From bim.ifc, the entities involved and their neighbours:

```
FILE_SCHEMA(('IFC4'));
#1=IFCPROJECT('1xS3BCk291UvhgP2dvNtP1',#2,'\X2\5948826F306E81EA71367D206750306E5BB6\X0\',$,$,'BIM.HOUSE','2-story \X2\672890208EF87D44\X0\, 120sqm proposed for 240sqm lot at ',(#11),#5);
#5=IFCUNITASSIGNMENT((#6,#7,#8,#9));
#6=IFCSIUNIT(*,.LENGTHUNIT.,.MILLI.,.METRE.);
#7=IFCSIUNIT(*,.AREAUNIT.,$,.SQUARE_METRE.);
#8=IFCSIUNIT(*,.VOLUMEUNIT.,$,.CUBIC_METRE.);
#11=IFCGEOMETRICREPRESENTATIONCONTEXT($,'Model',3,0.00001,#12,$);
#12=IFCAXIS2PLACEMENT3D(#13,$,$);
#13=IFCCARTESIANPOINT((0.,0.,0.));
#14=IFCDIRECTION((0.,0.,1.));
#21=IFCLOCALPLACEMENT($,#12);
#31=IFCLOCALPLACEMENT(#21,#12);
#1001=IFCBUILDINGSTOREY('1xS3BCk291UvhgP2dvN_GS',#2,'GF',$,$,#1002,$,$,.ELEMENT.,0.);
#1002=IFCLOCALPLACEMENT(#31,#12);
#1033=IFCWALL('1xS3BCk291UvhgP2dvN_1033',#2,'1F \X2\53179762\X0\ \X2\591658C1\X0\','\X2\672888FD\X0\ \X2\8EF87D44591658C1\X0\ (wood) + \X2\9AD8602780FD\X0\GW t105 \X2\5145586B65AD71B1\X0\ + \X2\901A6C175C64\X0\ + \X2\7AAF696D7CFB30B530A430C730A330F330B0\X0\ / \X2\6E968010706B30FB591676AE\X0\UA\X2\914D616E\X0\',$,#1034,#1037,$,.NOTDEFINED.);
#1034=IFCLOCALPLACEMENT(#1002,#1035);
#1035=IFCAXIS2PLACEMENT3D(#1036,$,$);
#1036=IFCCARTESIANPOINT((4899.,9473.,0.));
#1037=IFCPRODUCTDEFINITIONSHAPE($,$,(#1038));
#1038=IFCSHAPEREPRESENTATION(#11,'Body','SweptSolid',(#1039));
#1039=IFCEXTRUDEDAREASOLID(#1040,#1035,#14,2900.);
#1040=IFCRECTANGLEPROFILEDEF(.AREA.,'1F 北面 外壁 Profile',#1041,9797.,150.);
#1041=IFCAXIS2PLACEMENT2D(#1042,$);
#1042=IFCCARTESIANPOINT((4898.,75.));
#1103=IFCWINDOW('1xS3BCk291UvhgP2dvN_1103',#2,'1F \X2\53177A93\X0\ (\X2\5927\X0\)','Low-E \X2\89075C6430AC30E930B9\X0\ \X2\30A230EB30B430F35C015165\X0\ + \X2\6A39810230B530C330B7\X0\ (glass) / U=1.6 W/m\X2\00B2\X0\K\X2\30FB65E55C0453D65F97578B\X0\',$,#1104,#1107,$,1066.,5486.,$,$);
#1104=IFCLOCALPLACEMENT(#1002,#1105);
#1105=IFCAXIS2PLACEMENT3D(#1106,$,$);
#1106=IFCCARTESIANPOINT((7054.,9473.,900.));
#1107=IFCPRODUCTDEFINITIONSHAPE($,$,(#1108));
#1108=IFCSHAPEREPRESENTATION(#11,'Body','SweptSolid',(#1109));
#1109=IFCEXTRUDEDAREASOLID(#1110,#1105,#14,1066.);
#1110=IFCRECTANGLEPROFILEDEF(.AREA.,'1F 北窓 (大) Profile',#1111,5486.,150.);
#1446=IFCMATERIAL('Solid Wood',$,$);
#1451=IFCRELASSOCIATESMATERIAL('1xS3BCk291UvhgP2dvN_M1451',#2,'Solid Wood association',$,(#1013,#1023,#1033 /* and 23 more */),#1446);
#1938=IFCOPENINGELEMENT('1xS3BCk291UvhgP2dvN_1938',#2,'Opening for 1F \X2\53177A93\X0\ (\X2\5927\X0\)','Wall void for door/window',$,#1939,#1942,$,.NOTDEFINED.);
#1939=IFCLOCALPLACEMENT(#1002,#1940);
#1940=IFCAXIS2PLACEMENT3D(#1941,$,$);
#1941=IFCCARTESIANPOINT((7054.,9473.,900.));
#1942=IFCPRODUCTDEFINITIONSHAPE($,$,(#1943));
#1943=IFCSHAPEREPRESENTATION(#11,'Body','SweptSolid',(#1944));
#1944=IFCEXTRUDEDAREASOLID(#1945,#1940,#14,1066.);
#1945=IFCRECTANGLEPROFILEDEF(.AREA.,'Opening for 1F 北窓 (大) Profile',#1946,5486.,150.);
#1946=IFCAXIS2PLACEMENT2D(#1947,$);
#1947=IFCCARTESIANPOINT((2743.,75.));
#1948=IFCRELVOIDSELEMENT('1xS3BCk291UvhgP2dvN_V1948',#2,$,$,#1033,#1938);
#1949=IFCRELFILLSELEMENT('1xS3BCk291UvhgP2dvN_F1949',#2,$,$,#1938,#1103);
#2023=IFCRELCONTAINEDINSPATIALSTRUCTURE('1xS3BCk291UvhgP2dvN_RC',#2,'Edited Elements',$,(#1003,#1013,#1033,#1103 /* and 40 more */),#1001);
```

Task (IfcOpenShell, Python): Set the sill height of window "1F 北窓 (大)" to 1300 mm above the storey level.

```python
import numpy as np
import ifcopenshell
import ifcopenshell.api.geometry
import ifcopenshell.geom
import ifcopenshell.util.element
import ifcopenshell.util.placement
import ifcopenshell.util.shape
import ifcopenshell.util.unit

model = ifcopenshell.open("bim.ifc")
unit_scale = ifcopenshell.util.unit.calculate_unit_scale(model)

window = model.by_id(1103)
opening = window.FillsVoids[0].RelatingOpeningElement
storey = ifcopenshell.util.element.get_container(window, ifc_class="IfcBuildingStorey")
level = ifcopenshell.util.placement.get_local_placement(storey.ObjectPlacement)[2, 3]

# The opening's origin need not be at the sill, so measure its lowest point.
shape = ifcopenshell.geom.create_shape(ifcopenshell.geom.settings(), opening)
bottom = ifcopenshell.util.shape.get_shape_bottom_elevation(shape, shape.geometry) / unit_scale
dz = level + 1.3 / unit_scale - bottom

shift = np.array([0.0, 0.0, dz])
# The window is not placed relative to its opening, so move both.
for product in (opening, window):
    matrix = ifcopenshell.util.placement.get_local_placement(product.ObjectPlacement)
    matrix[:3, 3] += shift
    ifcopenshell.api.geometry.edit_object_placement(model, product=product, matrix=matrix, is_si=False)

print(f"moved by {dz * unit_scale:+.3f} m")

model.write("bim_v2.ifc")
```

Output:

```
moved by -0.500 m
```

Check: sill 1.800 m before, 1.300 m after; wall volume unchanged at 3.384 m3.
